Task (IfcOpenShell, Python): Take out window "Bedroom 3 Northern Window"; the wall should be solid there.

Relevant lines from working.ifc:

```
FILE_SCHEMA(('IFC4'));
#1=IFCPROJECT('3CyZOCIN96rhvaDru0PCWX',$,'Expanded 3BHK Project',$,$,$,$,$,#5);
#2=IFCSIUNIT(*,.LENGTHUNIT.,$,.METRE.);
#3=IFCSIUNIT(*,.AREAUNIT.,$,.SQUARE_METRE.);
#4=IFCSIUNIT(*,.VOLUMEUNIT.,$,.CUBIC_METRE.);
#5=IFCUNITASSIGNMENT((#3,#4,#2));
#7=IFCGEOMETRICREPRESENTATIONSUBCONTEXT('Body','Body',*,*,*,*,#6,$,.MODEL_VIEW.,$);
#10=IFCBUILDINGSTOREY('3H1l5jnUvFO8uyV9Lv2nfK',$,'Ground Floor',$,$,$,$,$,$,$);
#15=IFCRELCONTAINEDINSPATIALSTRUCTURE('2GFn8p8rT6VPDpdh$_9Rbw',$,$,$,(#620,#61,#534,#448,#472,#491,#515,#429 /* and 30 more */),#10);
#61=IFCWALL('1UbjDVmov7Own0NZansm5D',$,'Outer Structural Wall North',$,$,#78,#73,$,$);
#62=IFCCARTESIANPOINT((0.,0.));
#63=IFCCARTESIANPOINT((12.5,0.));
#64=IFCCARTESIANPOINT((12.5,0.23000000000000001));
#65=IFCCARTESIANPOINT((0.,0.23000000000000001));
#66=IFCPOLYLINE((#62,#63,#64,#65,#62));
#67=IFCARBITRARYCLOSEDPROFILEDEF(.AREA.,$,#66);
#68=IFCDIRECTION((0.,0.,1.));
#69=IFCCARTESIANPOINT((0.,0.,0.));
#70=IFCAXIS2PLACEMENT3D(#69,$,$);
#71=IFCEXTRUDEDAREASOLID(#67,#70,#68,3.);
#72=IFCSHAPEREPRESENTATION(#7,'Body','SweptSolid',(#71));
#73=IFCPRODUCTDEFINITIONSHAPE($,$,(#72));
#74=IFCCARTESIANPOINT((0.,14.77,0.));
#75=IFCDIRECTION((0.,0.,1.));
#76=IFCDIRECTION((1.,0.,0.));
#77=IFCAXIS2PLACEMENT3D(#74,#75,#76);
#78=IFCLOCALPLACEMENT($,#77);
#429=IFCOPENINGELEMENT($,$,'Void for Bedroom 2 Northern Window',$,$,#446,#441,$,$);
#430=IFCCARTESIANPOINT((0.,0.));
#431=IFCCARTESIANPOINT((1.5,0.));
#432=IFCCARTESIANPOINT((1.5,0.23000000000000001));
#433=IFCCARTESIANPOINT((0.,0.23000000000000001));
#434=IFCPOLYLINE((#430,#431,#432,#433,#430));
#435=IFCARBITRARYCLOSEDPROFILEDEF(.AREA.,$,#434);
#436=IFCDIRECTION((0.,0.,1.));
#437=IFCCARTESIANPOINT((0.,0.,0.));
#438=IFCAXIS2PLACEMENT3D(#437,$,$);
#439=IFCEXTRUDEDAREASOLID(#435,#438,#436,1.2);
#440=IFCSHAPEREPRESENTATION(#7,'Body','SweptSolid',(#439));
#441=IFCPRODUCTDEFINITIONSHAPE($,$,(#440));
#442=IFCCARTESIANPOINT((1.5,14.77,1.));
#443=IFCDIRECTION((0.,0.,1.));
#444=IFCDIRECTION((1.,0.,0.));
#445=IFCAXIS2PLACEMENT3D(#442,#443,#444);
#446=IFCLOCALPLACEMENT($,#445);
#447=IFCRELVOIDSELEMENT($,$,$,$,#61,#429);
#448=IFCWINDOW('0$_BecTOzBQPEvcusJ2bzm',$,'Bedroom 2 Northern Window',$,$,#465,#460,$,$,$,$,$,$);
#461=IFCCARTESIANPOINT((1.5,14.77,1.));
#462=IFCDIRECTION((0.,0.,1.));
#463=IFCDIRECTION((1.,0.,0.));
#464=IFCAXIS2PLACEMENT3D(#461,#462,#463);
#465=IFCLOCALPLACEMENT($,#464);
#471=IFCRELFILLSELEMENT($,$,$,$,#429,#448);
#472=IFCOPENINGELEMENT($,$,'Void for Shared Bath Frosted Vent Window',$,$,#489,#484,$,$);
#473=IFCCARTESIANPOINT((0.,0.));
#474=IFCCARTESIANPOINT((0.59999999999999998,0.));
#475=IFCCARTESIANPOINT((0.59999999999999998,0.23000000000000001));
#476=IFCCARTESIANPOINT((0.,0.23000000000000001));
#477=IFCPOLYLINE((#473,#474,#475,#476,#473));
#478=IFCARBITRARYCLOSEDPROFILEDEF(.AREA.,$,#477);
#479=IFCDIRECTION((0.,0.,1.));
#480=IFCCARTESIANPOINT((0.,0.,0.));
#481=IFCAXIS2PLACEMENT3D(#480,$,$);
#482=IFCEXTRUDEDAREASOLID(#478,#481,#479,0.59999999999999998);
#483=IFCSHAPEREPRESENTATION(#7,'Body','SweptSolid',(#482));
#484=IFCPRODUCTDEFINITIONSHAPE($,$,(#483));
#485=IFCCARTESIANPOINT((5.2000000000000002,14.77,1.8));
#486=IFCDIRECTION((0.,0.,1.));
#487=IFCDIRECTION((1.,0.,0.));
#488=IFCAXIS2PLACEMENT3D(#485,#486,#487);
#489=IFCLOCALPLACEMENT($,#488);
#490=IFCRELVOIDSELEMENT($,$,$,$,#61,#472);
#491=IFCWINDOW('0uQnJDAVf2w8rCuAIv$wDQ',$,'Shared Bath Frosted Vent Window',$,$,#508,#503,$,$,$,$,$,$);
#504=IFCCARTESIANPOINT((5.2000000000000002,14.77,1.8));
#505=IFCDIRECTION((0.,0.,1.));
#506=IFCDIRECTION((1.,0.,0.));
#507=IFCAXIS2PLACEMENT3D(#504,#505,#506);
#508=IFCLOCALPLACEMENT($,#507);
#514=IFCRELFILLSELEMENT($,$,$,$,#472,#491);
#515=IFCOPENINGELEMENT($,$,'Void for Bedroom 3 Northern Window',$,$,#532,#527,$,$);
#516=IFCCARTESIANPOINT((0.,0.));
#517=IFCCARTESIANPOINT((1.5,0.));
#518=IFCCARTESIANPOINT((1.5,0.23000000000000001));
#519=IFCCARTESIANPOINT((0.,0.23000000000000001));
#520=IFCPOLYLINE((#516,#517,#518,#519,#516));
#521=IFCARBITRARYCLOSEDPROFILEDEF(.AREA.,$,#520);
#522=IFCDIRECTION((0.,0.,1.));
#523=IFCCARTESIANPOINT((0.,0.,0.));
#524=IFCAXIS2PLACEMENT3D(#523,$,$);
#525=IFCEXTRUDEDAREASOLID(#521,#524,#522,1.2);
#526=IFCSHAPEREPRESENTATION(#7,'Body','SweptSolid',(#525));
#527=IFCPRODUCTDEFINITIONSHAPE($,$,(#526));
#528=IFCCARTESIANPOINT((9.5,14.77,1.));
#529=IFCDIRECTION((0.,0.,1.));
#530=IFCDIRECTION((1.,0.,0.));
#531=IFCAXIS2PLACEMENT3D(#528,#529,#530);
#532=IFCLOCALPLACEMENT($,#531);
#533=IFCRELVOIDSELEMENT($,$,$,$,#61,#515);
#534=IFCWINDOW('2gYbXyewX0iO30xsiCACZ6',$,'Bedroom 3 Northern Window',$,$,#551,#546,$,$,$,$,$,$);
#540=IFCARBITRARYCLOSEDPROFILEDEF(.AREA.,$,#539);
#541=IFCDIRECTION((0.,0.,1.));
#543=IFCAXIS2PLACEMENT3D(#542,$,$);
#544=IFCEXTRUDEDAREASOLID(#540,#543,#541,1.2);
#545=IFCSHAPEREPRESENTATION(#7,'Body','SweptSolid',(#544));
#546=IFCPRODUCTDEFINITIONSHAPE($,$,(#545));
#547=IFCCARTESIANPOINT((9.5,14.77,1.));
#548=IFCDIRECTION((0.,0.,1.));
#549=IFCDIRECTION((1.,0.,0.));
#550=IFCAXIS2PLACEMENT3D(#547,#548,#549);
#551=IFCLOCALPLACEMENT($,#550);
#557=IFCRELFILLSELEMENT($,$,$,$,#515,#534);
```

```python
import ifcopenshell
import ifcopenshell.api.feature
import ifcopenshell.api.root
import ifcopenshell.geom
import ifcopenshell.util.shape

model = ifcopenshell.open("working.ifc")
settings = ifcopenshell.geom.settings()


def volume(element):
    """Net volume in cubic metres, openings subtracted."""
    shape = ifcopenshell.geom.create_shape(settings, element)
    return ifcopenshell.util.shape.get_volume(shape.geometry)


window = model.by_guid("2gYbXyewX0iO30xsiCACZ6")
opening = window.FillsVoids[0].RelatingOpeningElement
wall = opening.VoidsElements[0].RelatingBuildingElement
before = volume(wall)

ifcopenshell.api.root.remove_product(model, product=window)
ifcopenshell.api.feature.remove_feature(model, feature=opening)

after = volume(wall)

print(f"wall volume {before:.3f} -> {after:.3f} m3")

model.write("working_v2.ifc")
```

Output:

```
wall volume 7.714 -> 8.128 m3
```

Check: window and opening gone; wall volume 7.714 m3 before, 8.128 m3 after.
